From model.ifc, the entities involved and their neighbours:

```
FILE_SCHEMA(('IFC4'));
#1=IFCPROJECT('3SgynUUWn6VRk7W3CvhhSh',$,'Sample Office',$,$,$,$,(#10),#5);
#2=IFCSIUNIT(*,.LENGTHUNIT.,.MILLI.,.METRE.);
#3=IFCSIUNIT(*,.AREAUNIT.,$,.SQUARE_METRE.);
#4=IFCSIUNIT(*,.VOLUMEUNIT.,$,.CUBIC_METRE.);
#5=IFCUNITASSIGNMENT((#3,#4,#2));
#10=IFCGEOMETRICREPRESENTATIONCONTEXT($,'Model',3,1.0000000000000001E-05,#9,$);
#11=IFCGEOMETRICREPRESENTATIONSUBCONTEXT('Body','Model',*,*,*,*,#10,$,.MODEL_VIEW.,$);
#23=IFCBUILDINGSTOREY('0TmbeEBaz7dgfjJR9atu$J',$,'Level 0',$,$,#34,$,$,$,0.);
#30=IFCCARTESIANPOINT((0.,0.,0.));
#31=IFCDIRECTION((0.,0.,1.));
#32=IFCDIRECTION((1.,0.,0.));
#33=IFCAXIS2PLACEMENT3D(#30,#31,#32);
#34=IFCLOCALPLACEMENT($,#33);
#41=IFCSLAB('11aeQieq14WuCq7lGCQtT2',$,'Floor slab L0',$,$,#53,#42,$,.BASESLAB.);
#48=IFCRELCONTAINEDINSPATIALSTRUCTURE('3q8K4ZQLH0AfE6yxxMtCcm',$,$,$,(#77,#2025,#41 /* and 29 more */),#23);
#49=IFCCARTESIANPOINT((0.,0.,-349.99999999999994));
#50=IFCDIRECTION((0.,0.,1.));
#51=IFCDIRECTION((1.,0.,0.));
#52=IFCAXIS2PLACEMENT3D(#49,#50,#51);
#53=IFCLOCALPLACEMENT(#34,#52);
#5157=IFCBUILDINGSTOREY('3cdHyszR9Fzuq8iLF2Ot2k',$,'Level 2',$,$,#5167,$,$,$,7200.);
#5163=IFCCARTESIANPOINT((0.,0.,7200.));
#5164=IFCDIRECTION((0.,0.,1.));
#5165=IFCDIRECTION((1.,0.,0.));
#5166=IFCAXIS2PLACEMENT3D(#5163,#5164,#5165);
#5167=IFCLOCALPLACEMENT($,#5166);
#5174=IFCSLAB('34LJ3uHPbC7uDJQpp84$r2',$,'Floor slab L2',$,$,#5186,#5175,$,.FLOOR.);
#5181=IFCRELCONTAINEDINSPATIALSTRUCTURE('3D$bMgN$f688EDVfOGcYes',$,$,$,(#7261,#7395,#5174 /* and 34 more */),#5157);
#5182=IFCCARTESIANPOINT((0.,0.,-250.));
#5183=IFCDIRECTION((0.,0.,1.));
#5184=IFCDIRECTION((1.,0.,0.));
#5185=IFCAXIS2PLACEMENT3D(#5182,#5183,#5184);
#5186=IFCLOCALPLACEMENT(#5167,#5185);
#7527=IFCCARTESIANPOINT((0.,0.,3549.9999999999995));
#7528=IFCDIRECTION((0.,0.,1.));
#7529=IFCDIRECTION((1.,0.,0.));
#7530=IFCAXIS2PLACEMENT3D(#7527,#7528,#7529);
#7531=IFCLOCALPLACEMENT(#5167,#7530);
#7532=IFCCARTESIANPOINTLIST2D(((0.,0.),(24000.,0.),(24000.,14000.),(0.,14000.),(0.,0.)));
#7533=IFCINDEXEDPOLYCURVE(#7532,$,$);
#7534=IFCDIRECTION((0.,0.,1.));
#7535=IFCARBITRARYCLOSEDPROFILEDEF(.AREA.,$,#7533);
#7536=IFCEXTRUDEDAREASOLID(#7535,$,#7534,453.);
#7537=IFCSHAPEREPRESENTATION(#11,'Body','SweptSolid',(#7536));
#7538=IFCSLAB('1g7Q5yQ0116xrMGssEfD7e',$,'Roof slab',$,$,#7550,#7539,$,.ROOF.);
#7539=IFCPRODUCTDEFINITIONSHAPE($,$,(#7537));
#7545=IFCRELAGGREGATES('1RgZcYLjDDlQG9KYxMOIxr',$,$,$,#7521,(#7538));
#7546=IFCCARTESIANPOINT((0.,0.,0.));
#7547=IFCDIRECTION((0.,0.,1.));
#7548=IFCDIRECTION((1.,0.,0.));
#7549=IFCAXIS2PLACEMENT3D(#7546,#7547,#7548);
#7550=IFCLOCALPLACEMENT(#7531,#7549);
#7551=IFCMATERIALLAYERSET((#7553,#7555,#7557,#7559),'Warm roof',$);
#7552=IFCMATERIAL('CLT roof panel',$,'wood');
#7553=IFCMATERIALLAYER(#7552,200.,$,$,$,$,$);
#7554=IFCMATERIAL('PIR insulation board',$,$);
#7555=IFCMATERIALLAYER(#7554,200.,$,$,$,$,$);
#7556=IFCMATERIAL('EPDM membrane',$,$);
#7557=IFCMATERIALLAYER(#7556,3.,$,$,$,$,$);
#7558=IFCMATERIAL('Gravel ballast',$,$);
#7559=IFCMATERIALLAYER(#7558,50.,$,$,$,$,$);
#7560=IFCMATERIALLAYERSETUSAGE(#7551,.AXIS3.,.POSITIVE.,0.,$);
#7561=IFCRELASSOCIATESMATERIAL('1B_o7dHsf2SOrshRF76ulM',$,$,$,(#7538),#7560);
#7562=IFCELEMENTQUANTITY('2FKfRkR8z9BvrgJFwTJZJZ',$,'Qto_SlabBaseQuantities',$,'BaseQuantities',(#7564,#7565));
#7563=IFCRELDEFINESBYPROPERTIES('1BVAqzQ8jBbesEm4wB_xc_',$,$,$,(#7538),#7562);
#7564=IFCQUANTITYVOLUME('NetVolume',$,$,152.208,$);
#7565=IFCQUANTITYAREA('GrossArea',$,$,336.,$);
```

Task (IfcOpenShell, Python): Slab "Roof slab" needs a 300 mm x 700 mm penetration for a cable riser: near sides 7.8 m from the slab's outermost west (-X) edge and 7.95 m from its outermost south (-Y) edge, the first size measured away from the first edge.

```python
import numpy as np
import ifcopenshell
import ifcopenshell.api.feature
import ifcopenshell.api.geometry
import ifcopenshell.api.pset
import ifcopenshell.api.root
import ifcopenshell.geom
import ifcopenshell.util.element
import ifcopenshell.util.placement
import ifcopenshell.util.representation
import ifcopenshell.util.shape
import ifcopenshell.util.unit

model = ifcopenshell.open("model.ifc")
unit_scale = ifcopenshell.util.unit.calculate_unit_scale(model)
volume_scale = ifcopenshell.util.unit.calculate_unit_scale(model, "VOLUMEUNIT")
settings = ifcopenshell.geom.settings()


def volume(element):
    """Net volume in cubic metres, openings subtracted."""
    shape = ifcopenshell.geom.create_shape(settings, element)
    return ifcopenshell.util.shape.get_volume(shape.geometry)


slab = model.by_guid("1g7Q5yQ0116xrMGssEfD7e")
before = volume(slab)

# Extent in the slab's own axes, in metres. The edges named are its -X and -Y sides.
slab_shape = ifcopenshell.geom.create_shape(settings, slab)
vertices = ifcopenshell.util.shape.get_vertices(slab_shape.geometry)
x_min, y_min, bottom = vertices.min(axis=0)
top = vertices[:, 2].max()

opening = ifcopenshell.api.root.create_entity(model, ifc_class="IfcOpeningElement", name="Cable riser opening", predefined_type="OPENING")
context = ifcopenshell.util.representation.get_context(model, "Model", "Body", "MODEL_VIEW")
width, depth = 0.3, 0.7
outline = [(0.0, 0.0), (width, 0.0), (width, depth), (0.0, depth), (0.0, 0.0)]
# Overshoot both faces by 50 mm so the cut is clean.
shape = ifcopenshell.api.geometry.add_slab_representation(
    model, context=context, depth=top - bottom + 0.1, polyline=outline
)
ifcopenshell.api.geometry.assign_representation(model, product=opening, representation=shape)

matrix = ifcopenshell.util.placement.get_local_placement(slab.ObjectPlacement)
matrix[:, 3] = matrix @ np.append(np.array([x_min + 7.8, y_min + 7.95, bottom - 0.05]) / unit_scale, 1.0)
ifcopenshell.api.geometry.edit_object_placement(model, product=opening, matrix=matrix, is_si=False)
ifcopenshell.api.feature.add_feature(model, feature=opening, element=slab)

after = volume(slab)

# Update the slab's stored quantities.
qto = model.by_id(ifcopenshell.util.element.get_pset(slab, "Qto_SlabBaseQuantities", should_inherit=False)["id"])
ifcopenshell.api.pset.edit_qto(model, qto=qto, properties={"NetVolume": after / volume_scale})

print(f"slab volume {before:.3f} -> {after:.3f} m3")

model.write("model-out.ifc")
```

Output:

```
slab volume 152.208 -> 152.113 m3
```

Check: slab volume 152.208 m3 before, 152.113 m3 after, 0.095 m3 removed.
